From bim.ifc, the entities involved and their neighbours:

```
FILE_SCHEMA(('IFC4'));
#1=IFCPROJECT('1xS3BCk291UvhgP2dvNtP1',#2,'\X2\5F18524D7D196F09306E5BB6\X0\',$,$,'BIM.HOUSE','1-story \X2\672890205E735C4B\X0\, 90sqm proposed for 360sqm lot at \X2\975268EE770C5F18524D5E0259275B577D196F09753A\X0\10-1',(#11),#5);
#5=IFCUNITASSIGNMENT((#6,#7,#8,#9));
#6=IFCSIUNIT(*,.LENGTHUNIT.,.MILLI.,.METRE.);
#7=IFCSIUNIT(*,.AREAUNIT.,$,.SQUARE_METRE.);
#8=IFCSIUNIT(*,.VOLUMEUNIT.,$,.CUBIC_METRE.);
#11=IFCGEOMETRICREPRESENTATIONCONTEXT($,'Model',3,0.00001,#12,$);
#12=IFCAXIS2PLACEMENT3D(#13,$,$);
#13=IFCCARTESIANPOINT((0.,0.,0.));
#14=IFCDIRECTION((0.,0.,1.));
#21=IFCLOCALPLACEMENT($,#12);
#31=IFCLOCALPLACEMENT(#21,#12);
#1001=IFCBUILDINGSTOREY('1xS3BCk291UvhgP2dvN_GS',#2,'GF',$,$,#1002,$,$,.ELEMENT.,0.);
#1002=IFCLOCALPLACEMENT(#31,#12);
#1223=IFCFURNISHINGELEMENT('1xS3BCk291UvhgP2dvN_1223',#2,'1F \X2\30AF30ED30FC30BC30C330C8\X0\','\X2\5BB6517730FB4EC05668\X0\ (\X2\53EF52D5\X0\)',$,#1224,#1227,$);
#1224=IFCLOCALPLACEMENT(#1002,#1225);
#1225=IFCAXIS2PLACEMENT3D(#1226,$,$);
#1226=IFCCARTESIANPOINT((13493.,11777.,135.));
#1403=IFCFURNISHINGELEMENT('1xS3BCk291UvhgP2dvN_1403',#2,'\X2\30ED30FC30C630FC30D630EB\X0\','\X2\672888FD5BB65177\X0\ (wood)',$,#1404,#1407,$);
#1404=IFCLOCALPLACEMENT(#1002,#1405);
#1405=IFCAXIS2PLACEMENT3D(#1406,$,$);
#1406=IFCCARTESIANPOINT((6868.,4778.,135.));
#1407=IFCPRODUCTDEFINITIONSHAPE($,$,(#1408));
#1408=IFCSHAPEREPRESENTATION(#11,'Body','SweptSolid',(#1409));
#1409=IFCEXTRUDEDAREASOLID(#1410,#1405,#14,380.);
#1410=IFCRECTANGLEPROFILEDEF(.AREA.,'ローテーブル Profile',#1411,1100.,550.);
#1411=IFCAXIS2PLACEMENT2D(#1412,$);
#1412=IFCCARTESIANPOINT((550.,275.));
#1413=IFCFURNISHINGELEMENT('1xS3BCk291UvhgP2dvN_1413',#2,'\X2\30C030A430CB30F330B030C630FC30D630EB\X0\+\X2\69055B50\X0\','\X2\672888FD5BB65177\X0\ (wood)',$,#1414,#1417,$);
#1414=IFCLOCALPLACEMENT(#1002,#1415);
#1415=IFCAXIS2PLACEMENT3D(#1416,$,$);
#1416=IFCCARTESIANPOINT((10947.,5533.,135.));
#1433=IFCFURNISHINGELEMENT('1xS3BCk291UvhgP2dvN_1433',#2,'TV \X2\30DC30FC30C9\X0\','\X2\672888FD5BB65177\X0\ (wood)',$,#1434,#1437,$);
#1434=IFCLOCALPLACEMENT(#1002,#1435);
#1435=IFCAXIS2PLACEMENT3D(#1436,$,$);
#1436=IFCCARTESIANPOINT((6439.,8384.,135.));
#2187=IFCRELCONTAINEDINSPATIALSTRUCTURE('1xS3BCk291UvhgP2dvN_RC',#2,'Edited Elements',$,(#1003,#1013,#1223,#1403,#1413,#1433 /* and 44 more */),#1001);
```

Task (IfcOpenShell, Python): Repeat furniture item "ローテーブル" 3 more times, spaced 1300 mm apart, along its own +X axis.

```python
import ifcopenshell
import ifcopenshell.api.geometry
import ifcopenshell.api.root
import ifcopenshell.util.element
import ifcopenshell.util.placement
import ifcopenshell.util.unit

model = ifcopenshell.open("bim.ifc")
unit_scale = ifcopenshell.util.unit.calculate_unit_scale(model)


def reuse_history(source, copy):
    """copy_class also copies each property set's owner history, people and application; keep the originals."""
    for rel in copy.IsDefinedBy:
        if rel.is_a("IfcRelDefinesByProperties") and (history := rel.RelatingPropertyDefinition.OwnerHistory):
            rel.RelatingPropertyDefinition.OwnerHistory = source.OwnerHistory
            ifcopenshell.util.element.remove_deep2(model, history)


source = model.by_guid("1xS3BCk291UvhgP2dvN_1403")
base = ifcopenshell.util.placement.get_local_placement(source.ObjectPlacement)
step = base[:3, 0] * 1.3 / unit_scale

for i in range(1, 4):
    copy = ifcopenshell.api.root.copy_class(model, product=source)
    copy.Representation = ifcopenshell.util.element.copy_deep(
        model, source.Representation, exclude=["IfcGeometricRepresentationContext", "IfcRepresentationMap"]
    )
    reuse_history(source, copy)
    matrix = base.copy()
    matrix[:3, 3] += i * step
    print("added at", matrix[:3, 3].round(3) + 0.0)
    ifcopenshell.api.geometry.edit_object_placement(model, product=copy, matrix=matrix, is_si=False)

model.write("bim_updated.ifc")
```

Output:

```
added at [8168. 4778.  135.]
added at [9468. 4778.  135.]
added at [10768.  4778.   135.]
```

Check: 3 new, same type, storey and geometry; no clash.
